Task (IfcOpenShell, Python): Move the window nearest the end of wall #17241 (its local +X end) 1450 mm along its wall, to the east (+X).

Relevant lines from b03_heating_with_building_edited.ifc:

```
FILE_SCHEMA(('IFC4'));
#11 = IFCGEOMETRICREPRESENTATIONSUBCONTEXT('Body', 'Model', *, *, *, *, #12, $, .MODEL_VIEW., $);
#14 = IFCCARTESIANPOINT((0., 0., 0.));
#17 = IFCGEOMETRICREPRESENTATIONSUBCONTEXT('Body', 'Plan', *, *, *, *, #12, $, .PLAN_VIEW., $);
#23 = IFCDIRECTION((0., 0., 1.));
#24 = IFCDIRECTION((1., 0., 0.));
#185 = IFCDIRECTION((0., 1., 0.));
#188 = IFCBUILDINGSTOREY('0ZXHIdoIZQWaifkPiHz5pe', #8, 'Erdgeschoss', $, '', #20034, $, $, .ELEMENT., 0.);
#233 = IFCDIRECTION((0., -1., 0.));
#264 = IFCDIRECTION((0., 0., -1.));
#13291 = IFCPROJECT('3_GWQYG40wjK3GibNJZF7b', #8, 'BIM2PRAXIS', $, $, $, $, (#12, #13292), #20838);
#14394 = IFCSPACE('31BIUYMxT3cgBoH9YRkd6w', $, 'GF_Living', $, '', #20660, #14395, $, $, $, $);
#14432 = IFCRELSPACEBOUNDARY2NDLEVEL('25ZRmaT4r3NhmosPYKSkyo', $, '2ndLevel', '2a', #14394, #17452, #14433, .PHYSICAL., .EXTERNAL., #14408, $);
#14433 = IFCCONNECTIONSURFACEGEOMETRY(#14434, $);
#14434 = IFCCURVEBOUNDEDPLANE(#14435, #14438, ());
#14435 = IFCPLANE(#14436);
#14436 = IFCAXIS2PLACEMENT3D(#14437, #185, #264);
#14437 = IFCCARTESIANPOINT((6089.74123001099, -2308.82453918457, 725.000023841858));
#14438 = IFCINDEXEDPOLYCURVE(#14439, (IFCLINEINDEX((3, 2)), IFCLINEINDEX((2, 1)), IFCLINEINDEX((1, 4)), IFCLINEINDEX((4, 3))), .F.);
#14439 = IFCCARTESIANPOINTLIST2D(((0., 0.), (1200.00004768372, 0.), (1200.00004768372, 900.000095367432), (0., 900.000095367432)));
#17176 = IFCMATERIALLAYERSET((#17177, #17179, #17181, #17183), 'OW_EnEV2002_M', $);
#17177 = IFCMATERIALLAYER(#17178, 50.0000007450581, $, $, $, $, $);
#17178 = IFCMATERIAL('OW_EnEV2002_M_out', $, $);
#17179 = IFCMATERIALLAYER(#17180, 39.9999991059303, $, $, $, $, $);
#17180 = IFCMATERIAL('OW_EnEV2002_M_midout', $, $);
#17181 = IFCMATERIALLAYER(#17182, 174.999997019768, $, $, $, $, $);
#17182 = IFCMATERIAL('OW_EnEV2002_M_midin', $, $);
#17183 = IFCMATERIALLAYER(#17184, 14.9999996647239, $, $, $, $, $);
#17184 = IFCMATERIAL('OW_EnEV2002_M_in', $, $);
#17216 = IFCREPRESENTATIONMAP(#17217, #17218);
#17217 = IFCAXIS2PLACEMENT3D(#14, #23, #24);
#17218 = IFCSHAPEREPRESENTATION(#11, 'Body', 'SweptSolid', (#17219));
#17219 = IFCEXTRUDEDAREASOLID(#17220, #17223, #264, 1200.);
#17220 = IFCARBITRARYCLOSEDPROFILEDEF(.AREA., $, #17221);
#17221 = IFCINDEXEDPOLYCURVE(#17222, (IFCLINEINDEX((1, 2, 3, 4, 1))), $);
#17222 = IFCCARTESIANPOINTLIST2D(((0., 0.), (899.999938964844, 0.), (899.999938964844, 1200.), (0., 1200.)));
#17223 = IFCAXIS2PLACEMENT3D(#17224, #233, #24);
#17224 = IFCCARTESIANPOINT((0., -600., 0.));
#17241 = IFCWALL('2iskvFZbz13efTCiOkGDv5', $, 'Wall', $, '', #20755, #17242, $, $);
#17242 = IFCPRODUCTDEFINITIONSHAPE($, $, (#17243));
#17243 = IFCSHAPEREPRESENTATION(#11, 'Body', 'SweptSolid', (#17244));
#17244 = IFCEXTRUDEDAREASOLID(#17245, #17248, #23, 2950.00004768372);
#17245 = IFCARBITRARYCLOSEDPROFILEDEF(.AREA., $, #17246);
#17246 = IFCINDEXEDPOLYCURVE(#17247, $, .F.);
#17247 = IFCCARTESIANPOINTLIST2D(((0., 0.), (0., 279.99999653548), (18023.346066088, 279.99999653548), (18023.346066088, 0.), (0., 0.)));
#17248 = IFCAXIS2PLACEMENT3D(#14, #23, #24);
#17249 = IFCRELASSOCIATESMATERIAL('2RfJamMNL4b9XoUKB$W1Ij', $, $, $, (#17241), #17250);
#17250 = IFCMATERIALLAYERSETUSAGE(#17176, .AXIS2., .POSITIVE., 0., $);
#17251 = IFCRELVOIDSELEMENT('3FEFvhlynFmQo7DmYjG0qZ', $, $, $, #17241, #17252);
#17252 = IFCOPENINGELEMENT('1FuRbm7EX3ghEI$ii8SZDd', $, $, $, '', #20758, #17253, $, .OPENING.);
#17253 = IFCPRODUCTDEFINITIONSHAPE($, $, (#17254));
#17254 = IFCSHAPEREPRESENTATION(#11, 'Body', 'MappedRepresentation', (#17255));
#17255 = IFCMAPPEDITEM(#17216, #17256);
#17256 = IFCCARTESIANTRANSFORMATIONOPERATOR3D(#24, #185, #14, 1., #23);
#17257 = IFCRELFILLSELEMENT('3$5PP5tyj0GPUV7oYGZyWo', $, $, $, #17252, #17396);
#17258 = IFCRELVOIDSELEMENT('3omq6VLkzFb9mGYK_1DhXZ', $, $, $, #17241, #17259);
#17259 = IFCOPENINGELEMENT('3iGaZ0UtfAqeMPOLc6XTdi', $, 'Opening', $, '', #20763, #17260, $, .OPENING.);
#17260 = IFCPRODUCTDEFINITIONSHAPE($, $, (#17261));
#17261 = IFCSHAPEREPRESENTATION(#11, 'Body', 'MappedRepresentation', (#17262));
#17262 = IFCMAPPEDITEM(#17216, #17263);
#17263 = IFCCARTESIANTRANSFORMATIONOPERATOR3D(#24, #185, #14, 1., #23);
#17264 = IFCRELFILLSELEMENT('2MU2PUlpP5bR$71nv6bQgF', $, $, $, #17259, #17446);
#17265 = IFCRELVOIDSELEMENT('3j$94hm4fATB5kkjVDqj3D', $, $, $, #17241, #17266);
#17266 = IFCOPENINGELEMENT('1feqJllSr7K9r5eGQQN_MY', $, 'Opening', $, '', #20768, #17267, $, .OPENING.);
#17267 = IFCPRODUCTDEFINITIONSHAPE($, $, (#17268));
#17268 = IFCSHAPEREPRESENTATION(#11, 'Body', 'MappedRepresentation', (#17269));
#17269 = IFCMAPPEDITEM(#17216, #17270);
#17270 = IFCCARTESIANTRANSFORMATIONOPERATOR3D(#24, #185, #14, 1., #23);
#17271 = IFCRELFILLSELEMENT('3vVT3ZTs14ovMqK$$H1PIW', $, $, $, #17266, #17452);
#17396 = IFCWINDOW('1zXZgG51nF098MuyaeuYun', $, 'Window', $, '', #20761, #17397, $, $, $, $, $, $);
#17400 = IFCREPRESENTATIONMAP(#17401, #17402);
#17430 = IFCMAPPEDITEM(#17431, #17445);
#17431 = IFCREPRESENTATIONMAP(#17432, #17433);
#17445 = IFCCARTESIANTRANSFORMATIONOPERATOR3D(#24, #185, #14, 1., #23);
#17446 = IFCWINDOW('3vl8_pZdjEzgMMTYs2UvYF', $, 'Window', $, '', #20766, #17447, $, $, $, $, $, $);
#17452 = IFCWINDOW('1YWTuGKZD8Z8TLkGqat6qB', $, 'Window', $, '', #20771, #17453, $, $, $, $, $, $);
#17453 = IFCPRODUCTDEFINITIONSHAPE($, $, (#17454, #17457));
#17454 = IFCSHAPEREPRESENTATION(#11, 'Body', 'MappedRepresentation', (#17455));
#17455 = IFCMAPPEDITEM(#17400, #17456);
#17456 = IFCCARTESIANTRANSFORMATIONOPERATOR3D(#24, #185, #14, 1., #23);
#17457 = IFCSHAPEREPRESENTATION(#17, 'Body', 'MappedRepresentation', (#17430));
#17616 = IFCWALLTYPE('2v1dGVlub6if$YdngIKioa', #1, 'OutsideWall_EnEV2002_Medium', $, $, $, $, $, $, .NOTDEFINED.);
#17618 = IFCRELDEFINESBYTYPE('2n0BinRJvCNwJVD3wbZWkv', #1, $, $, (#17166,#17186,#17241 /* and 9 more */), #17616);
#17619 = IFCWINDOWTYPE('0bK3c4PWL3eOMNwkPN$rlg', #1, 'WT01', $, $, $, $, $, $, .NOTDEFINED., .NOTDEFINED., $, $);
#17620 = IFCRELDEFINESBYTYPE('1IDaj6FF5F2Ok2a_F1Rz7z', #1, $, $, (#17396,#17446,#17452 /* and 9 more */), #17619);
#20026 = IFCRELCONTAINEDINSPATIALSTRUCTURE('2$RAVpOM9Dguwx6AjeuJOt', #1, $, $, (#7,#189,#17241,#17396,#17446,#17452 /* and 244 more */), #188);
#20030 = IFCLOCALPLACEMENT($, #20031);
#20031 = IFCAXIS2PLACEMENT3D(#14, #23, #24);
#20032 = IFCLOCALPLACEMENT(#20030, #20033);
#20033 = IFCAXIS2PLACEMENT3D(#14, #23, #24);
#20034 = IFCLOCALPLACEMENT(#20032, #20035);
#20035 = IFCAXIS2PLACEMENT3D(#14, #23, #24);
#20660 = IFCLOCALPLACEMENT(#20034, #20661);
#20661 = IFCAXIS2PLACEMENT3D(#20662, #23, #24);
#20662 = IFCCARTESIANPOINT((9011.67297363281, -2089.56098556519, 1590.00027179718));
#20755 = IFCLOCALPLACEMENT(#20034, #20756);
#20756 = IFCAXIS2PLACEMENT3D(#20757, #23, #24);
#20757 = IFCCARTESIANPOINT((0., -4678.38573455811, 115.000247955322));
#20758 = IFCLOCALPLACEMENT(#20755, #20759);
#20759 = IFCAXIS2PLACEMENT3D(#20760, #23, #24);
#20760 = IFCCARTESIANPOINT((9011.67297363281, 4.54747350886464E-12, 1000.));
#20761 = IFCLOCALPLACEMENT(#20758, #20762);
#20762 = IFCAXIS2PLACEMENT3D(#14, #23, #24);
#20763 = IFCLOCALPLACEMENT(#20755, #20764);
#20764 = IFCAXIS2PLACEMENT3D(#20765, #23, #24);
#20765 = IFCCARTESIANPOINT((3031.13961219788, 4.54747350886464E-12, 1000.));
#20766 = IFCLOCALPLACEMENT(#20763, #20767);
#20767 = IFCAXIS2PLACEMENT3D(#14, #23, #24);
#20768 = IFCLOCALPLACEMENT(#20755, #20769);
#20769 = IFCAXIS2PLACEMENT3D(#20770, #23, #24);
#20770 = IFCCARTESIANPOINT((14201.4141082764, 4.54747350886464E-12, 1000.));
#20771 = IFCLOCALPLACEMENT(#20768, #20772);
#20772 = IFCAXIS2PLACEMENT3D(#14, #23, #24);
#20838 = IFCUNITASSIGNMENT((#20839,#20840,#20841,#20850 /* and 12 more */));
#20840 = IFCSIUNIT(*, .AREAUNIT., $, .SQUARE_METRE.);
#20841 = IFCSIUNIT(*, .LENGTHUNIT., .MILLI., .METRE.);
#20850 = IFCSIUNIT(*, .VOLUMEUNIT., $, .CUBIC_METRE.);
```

```python
import numpy as np
import ifcopenshell
import ifcopenshell.api.geometry
import ifcopenshell.util.placement
import ifcopenshell.util.unit

model = ifcopenshell.open("b03_heating_with_building_edited.ifc")
unit_scale = ifcopenshell.util.unit.calculate_unit_scale(model)

window = model.by_id(17452)
opening = window.FillsVoids[0].RelatingOpeningElement
wall = opening.VoidsElements[0].RelatingBuildingElement

wall_matrix = ifcopenshell.util.placement.get_local_placement(wall.ObjectPlacement)
shift = wall_matrix[:3, 0] * 1.45 / unit_scale
before = ifcopenshell.util.placement.get_local_placement(window.ObjectPlacement)[:3, 3].copy()

# The window is placed relative to its opening, so it follows when the opening moves.
matrix = ifcopenshell.util.placement.get_local_placement(opening.ObjectPlacement)
matrix[:3, 3] += shift
ifcopenshell.api.geometry.edit_object_placement(
    model, product=opening, matrix=matrix, is_si=False, should_transform_children=True
)

# Space boundary surfaces are stored in each space's coordinates; move them too.
for rel in window.ProvidesBoundaries:
    if not rel.ConnectionGeometry:
        continue
    surface = rel.ConnectionGeometry.SurfaceOnRelatingElement.BasisSurface
    space_matrix = ifcopenshell.util.placement.get_local_placement(rel.RelatingSpace.ObjectPlacement)
    point = np.array(surface.Position.Location.Coordinates) + space_matrix[:3, :3].T @ shift
    surface.Position = model.createIfcAxis2Placement3D(
        model.createIfcCartesianPoint(point.tolist()), surface.Position.Axis, surface.Position.RefDirection
    )

after = ifcopenshell.util.placement.get_local_placement(window.ObjectPlacement)[:3, 3]
print("window moved by", (after - before).round(3) + 0.0)

model.write("b03_heating_with_building_edited_updated.ifc")
```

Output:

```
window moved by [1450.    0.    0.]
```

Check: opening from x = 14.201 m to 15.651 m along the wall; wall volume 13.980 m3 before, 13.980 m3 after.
